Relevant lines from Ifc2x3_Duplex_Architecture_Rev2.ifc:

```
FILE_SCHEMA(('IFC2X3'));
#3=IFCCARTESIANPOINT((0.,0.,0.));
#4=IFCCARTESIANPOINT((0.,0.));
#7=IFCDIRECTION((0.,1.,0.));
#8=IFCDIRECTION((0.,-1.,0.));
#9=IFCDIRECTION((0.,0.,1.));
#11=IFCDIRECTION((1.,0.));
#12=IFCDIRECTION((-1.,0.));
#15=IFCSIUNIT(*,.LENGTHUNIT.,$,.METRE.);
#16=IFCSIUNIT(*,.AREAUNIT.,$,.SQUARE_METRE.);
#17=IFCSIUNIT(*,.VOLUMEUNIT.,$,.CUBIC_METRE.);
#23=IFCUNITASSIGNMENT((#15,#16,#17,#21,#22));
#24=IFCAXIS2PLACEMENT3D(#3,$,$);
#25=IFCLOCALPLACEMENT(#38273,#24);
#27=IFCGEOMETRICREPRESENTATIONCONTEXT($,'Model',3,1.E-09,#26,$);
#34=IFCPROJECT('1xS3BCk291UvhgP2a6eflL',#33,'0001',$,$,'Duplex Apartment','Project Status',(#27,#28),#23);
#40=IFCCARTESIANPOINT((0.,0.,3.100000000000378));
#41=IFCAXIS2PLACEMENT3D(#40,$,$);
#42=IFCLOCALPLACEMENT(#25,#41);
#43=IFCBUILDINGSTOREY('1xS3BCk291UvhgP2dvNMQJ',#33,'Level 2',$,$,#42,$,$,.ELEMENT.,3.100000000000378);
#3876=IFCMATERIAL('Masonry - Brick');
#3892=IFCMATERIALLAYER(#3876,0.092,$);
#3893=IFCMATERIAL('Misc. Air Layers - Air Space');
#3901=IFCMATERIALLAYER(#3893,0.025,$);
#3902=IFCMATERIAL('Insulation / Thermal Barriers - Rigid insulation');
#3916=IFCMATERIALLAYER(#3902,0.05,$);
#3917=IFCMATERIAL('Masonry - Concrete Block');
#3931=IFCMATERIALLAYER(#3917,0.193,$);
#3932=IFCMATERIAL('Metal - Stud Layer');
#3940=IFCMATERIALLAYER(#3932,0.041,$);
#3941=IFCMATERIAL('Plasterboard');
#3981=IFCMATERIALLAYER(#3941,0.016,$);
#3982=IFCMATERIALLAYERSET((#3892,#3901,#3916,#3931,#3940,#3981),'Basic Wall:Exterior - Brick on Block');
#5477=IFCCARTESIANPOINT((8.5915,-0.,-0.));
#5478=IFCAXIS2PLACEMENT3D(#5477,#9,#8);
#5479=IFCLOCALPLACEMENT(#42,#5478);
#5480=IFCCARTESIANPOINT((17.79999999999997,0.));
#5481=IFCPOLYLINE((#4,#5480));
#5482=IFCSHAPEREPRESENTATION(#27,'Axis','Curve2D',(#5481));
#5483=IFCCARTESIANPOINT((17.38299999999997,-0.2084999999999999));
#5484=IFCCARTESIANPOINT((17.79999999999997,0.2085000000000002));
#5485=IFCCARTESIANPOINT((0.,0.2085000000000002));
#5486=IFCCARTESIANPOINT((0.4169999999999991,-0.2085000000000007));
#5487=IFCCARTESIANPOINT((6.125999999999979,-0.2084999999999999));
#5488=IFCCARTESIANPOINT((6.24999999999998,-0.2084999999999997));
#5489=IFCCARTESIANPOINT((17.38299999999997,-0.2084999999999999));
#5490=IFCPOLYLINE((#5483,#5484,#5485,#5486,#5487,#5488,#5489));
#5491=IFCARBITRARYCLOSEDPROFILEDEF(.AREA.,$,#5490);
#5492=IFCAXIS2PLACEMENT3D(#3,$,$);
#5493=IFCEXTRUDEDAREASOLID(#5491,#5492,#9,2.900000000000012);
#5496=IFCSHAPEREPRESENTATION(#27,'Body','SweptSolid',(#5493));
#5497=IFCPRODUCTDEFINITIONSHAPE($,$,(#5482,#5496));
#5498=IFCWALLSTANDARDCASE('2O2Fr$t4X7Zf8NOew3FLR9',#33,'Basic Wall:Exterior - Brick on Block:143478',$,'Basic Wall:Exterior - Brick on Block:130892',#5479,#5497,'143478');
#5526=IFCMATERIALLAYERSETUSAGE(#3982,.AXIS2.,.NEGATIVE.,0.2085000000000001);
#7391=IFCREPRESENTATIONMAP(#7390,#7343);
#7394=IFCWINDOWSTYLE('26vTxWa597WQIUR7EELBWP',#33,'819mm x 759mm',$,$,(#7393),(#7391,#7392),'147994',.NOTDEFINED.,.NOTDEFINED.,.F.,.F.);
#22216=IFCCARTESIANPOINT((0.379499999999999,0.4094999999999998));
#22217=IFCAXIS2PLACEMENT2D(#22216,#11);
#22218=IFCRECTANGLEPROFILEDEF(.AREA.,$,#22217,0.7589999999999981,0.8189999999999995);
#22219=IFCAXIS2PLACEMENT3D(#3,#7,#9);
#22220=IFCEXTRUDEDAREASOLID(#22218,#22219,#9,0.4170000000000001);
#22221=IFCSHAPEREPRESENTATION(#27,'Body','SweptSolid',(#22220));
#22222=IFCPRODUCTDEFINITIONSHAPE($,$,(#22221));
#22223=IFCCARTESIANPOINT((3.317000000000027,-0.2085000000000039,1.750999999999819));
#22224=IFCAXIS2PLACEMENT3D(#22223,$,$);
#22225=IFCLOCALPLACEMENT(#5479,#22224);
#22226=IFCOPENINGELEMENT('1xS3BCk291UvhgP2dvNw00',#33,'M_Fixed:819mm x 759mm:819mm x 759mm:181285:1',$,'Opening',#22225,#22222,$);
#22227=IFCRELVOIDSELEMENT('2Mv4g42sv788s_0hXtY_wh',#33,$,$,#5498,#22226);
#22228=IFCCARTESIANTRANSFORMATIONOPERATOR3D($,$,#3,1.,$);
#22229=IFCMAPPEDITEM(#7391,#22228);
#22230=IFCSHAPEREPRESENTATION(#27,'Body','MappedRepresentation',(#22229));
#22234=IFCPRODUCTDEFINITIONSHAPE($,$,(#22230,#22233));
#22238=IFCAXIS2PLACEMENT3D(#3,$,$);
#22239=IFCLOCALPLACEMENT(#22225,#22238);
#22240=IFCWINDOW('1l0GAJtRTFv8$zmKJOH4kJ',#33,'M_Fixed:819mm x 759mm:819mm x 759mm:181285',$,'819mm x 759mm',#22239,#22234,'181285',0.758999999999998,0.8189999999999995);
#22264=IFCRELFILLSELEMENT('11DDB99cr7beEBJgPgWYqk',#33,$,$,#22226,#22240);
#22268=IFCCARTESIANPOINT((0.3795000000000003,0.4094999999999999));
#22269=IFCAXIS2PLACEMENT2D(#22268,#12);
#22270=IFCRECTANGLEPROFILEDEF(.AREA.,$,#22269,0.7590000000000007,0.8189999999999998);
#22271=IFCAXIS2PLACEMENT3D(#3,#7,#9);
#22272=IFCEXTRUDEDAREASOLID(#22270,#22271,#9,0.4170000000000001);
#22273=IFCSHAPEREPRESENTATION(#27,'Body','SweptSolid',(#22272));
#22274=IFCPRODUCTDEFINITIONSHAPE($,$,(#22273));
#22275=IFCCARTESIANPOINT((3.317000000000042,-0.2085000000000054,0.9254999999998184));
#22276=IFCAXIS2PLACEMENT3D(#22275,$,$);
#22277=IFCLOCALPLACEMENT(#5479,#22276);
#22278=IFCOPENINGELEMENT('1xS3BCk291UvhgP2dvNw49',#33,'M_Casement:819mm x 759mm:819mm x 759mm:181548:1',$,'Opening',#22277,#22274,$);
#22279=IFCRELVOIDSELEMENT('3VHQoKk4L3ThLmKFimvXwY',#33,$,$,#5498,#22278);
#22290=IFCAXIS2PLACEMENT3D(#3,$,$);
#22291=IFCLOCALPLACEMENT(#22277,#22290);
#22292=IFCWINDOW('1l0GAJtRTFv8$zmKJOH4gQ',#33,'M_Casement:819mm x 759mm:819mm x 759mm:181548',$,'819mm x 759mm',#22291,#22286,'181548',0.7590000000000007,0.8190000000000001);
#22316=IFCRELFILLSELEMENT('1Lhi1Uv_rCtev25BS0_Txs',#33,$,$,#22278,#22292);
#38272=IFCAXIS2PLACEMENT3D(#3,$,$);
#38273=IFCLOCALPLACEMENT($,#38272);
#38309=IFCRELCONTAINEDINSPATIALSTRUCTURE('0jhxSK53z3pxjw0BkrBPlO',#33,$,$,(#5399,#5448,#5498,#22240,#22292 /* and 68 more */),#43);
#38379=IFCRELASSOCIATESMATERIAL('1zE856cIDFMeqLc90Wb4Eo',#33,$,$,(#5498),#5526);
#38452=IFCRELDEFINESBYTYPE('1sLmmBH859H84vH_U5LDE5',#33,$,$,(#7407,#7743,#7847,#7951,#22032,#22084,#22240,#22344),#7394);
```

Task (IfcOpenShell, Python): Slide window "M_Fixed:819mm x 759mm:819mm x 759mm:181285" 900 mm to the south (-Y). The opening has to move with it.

```python
import ifcopenshell
import ifcopenshell.api.geometry
import ifcopenshell.util.placement

model = ifcopenshell.open("Ifc2x3_Duplex_Architecture_Rev2.ifc")

window = model.by_guid("1l0GAJtRTFv8$zmKJOH4kJ")
opening = window.FillsVoids[0].RelatingOpeningElement
wall = opening.VoidsElements[0].RelatingBuildingElement

wall_matrix = ifcopenshell.util.placement.get_local_placement(wall.ObjectPlacement)
shift = wall_matrix[:3, 0] * 0.9
before = ifcopenshell.util.placement.get_local_placement(window.ObjectPlacement)[:3, 3].copy()

# The window is placed relative to its opening, so it follows when the opening moves.
matrix = ifcopenshell.util.placement.get_local_placement(opening.ObjectPlacement)
matrix[:3, 3] += shift
ifcopenshell.api.geometry.edit_object_placement(
    model, product=opening, matrix=matrix, is_si=False, should_transform_children=True
)

after = ifcopenshell.util.placement.get_local_placement(window.ObjectPlacement)[:3, 3]
print("window moved by", (after - before).round(3) + 0.0)

model.write("Ifc2x3_Duplex_Architecture_Rev2_v2.ifc")
```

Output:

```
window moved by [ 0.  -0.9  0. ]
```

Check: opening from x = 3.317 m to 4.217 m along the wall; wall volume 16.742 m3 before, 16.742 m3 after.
